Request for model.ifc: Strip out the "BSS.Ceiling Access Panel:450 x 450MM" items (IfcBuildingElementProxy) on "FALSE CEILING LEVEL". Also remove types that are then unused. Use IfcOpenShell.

First a look at what the model holds.

```python
import ifcopenshell
import ifcopenshell.util.element

model = ifcopenshell.open("model.ifc")
print(model.schema)
storey = next(s for s in model.by_type("IfcBuildingStorey") if s.Name == "FALSE CEILING LEVEL")
proxies = [e for e in ifcopenshell.util.element.get_decomposition(storey) if e.is_a("IfcBuildingElementProxy")]
seen = {}
for e in proxies:
    element_type = ifcopenshell.util.element.get_type(e)
    name = element_type.Name if element_type not in (None, e) else None
    seen[name] = seen.get(name, 0) + 1
for name, count in sorted(seen.items(), key=str):
    print(count, "x", name)
```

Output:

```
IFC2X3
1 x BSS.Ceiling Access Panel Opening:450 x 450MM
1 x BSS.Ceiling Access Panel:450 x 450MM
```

```python
import ifcopenshell
import ifcopenshell.api.root
import ifcopenshell.util.element

model = ifcopenshell.open("model.ifc")

storey = next(s for s in model.by_type("IfcBuildingStorey") if s.Name == "FALSE CEILING LEVEL")
proxies = [e for e in ifcopenshell.util.element.get_decomposition(storey) if e.is_a("IfcBuildingElementProxy")]
targets = [e for e in proxies if (t := ifcopenshell.util.element.get_type(e)) not in (None, e) and t.Name == "BSS.Ceiling Access Panel:450 x 450MM"]
types = {ifcopenshell.util.element.get_type(e) for e in targets} - {None, *targets}

for e in targets:
    ifcopenshell.api.root.remove_product(model, product=e)
print(len(targets), "removed")

unused = [t for t in types if not ifcopenshell.util.element.get_types(t)]
for t in unused:
    ifcopenshell.api.root.remove_product(model, product=t)
print(len(unused), "unused types removed")

model.write("model_v2.ifc")
```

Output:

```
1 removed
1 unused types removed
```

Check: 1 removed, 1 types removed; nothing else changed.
